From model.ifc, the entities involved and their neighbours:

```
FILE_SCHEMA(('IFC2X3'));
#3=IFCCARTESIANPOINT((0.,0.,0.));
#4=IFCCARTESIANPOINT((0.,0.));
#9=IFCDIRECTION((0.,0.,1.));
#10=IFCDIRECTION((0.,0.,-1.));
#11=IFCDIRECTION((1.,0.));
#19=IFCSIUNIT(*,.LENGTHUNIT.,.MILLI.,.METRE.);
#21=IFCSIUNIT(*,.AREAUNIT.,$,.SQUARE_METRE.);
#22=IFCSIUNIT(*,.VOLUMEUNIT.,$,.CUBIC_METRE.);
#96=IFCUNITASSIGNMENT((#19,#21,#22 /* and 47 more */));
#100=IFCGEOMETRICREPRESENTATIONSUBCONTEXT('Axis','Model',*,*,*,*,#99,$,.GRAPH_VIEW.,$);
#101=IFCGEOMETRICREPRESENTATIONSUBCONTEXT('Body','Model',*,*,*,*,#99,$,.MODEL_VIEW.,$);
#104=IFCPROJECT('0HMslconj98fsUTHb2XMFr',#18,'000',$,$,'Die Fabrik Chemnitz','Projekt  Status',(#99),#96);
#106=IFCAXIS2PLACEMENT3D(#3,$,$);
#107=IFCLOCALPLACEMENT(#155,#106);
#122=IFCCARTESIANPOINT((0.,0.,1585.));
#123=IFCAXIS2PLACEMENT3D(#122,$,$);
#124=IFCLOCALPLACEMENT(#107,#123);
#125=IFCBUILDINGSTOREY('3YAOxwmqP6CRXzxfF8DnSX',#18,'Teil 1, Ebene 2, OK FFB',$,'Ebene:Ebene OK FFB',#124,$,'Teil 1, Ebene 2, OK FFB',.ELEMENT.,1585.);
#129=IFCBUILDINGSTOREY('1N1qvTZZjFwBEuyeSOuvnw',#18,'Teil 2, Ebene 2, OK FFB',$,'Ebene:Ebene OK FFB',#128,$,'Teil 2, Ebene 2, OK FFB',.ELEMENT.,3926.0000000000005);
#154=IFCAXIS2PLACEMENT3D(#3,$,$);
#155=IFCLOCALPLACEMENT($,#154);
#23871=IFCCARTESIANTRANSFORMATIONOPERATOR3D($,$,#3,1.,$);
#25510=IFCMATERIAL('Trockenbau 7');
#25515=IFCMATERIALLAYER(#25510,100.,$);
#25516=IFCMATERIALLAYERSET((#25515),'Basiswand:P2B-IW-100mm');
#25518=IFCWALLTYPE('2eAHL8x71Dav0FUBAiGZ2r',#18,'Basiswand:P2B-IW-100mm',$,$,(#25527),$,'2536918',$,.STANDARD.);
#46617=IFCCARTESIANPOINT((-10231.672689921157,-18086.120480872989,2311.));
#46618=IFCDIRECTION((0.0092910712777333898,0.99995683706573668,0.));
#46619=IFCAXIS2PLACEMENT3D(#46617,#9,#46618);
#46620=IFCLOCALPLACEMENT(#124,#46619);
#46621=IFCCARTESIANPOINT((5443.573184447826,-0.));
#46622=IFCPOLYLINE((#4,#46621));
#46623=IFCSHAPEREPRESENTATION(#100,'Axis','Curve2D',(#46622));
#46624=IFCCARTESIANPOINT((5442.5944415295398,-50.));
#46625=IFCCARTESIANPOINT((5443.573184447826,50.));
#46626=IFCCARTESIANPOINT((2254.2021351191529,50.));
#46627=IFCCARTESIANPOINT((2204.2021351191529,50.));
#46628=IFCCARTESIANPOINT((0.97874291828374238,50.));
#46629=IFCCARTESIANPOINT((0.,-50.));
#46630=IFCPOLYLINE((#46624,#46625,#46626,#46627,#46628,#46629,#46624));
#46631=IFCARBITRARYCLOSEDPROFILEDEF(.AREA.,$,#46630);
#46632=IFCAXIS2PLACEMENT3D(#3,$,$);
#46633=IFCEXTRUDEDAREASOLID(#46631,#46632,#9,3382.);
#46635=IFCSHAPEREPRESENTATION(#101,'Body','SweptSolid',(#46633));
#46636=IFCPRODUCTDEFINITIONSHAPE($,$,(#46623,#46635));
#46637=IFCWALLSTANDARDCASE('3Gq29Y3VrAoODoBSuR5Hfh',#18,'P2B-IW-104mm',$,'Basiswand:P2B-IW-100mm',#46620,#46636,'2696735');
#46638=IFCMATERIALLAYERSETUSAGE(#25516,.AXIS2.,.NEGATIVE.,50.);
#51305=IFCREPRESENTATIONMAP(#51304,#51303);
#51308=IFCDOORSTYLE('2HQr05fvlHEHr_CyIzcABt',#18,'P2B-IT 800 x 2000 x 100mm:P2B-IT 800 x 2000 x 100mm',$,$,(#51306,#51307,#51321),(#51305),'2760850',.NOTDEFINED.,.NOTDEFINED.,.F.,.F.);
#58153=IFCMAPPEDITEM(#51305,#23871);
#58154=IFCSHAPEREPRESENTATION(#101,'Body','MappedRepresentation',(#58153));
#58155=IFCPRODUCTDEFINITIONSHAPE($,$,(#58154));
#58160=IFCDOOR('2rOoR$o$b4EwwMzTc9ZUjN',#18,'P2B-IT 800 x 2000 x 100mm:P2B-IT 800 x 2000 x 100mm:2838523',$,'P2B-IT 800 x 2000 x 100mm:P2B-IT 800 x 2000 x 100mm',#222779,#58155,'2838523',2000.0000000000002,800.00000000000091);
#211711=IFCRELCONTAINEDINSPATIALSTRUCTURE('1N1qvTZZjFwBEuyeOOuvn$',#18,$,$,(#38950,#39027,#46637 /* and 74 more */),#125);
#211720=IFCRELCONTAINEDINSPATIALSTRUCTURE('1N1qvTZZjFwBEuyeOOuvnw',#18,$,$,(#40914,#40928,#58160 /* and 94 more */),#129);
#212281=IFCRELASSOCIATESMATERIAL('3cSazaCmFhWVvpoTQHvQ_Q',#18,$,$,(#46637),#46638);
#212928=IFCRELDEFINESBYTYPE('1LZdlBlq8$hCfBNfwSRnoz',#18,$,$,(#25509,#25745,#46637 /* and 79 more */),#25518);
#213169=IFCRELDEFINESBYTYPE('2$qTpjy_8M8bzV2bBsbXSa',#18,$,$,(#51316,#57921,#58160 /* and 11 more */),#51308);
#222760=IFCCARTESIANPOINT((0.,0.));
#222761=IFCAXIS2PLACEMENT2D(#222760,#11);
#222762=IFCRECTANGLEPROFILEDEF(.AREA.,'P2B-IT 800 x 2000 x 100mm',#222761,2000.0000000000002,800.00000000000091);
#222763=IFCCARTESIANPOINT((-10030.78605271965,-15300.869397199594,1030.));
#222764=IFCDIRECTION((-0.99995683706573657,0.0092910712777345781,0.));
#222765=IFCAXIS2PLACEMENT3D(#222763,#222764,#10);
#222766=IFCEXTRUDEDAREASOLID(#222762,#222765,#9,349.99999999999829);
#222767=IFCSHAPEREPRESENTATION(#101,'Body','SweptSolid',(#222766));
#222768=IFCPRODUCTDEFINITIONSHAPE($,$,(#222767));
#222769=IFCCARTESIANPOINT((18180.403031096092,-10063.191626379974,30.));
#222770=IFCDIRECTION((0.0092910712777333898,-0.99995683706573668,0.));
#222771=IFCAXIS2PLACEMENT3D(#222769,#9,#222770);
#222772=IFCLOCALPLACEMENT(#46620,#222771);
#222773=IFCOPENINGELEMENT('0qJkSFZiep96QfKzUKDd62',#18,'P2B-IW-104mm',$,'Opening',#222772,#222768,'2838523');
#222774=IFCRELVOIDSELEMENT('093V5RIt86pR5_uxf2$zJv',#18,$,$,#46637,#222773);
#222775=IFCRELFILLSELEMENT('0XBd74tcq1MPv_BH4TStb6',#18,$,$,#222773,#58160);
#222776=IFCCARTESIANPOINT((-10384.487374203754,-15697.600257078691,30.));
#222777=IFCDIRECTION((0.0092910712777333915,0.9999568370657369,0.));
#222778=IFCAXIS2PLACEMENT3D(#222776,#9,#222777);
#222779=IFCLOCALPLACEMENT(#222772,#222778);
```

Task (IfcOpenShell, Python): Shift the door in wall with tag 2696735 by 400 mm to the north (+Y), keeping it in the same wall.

```python
import ifcopenshell
import ifcopenshell.api.geometry
import ifcopenshell.util.placement

model = ifcopenshell.open("model.ifc")

door = model.by_id(58160)
opening = door.FillsVoids[0].RelatingOpeningElement
wall = opening.VoidsElements[0].RelatingBuildingElement

wall_matrix = ifcopenshell.util.placement.get_local_placement(wall.ObjectPlacement)
shift = wall_matrix[:3, 0] * 400.0
before = ifcopenshell.util.placement.get_local_placement(door.ObjectPlacement)[:3, 3].copy()

# The door is placed relative to its opening, so it follows when the opening moves.
matrix = ifcopenshell.util.placement.get_local_placement(opening.ObjectPlacement)
matrix[:3, 3] += shift
ifcopenshell.api.geometry.edit_object_placement(
    model, product=opening, matrix=matrix, is_si=False, should_transform_children=True
)

after = ifcopenshell.util.placement.get_local_placement(door.ObjectPlacement)[:3, 3]
print("door moved by", (after - before).round(3) + 0.0)

model.write("model_edited.ifc")
```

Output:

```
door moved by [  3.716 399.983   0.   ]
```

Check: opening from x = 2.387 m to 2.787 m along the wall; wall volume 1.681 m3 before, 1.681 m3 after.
